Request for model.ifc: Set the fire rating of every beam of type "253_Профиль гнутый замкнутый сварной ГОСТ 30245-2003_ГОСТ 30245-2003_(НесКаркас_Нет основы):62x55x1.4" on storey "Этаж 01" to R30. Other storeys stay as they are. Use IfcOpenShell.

First a look at what the model holds.

```python
import ifcopenshell
import ifcopenshell.util.element

model = ifcopenshell.open("model.ifc")
print(model.schema)
storey = next(s for s in model.by_type("IfcBuildingStorey") if s.Name == "Этаж 01")
beams = [e for e in ifcopenshell.util.element.get_decomposition(storey) if e.is_a("IfcBeam")]
seen = {}
for e in beams:
    element_type = ifcopenshell.util.element.get_type(e)
    key = (element_type.Name if element_type != e and element_type else None, ifcopenshell.util.element.get_pset(e, "Pset_BeamCommon", "FireRating"))
    seen[key] = seen.get(key, 0) + 1
for (name, value), count in sorted(seen.items(), key=str):
    print(count, "x", name, "|", value)
```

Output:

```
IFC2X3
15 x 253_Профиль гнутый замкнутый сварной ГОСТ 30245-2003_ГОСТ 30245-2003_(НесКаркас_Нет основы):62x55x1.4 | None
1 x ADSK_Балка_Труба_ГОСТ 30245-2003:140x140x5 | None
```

```python
import ifcopenshell
import ifcopenshell.api.pset
import ifcopenshell.util.element

model = ifcopenshell.open("model.ifc")

storey = next(s for s in model.by_type("IfcBuildingStorey") if s.Name == "Этаж 01")
beams = [e for e in ifcopenshell.util.element.get_decomposition(storey) if e.is_a("IfcBeam")]

count = 0
for e in beams:
    element_type = ifcopenshell.util.element.get_type(e)
    if element_type in (None, e) or element_type.Name != "253_Профиль гнутый замкнутый сварной ГОСТ 30245-2003_ГОСТ 30245-2003_(НесКаркас_Нет основы):62x55x1.4":
        continue
    # add_pset returns the element's existing set when there is one.
    pset = ifcopenshell.api.pset.add_pset(model, product=e, name="Pset_BeamCommon")
    ifcopenshell.api.pset.edit_pset(model, pset=pset, properties={"FireRating": "R30"})
    count += 1

print(count, "beams updated")

model.write("model_v2.ifc")
```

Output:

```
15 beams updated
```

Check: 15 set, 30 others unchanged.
